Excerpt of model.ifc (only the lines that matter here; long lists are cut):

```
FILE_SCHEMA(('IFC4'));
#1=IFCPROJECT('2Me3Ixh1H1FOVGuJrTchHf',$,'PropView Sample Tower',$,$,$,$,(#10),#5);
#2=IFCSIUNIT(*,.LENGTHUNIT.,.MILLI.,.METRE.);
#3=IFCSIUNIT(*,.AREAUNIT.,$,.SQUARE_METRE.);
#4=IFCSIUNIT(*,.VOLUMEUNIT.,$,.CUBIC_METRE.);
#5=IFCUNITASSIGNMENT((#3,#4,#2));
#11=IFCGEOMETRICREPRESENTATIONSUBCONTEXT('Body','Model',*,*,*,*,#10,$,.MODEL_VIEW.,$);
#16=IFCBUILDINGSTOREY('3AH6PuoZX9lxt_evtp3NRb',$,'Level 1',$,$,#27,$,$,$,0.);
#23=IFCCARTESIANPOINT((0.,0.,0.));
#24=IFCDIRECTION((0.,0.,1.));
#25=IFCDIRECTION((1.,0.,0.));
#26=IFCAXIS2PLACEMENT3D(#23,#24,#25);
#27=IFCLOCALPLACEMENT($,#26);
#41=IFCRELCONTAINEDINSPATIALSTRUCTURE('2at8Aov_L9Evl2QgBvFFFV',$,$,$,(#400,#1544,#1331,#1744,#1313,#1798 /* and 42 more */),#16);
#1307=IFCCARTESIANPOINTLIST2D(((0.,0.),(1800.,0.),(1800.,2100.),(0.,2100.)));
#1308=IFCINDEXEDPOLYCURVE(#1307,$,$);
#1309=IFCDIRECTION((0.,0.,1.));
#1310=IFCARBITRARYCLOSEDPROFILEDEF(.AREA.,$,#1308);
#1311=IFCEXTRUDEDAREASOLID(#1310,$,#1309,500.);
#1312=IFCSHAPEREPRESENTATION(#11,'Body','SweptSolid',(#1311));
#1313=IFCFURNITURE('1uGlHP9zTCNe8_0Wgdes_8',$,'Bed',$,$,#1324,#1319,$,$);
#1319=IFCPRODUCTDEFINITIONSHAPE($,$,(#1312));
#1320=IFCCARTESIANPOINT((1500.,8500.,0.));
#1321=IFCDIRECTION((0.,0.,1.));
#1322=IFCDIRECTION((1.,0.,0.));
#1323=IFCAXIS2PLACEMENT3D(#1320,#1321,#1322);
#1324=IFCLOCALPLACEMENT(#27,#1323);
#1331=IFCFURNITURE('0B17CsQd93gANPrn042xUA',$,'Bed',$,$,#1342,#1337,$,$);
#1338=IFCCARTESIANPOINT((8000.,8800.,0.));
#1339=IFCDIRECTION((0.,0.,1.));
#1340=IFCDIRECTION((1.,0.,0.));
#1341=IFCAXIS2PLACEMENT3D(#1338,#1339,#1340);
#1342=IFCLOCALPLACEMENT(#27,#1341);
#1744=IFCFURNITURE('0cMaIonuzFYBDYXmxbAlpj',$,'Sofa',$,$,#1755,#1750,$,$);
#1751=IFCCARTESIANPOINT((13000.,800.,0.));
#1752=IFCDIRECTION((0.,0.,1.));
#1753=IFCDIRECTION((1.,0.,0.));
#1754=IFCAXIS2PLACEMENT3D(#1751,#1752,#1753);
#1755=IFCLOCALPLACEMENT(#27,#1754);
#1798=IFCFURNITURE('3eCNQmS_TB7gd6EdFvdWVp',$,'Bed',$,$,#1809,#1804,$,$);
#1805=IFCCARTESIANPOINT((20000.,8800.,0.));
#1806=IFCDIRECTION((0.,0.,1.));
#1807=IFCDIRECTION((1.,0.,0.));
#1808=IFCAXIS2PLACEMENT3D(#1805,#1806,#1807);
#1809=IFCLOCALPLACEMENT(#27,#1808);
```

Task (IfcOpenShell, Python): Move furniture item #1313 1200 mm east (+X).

```python
import ifcopenshell
import ifcopenshell.api.geometry
import ifcopenshell.util.placement
import ifcopenshell.util.unit

model = ifcopenshell.open("model.ifc")
unit_scale = ifcopenshell.util.unit.calculate_unit_scale(model)

item = model.by_guid("1uGlHP9zTCNe8_0Wgdes_8")
matrix = ifcopenshell.util.placement.get_local_placement(item.ObjectPlacement)
matrix[0, 3] += 1.2 / unit_scale
ifcopenshell.api.geometry.edit_object_placement(model, product=item, matrix=matrix, is_si=False)

print(ifcopenshell.util.placement.get_local_placement(item.ObjectPlacement).round(3) + 0.0)

model.write("model_edited.ifc")
```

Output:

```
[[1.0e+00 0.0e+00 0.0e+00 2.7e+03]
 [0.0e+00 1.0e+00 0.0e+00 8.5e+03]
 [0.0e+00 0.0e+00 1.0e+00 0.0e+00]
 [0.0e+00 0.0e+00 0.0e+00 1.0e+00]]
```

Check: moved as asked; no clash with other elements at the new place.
